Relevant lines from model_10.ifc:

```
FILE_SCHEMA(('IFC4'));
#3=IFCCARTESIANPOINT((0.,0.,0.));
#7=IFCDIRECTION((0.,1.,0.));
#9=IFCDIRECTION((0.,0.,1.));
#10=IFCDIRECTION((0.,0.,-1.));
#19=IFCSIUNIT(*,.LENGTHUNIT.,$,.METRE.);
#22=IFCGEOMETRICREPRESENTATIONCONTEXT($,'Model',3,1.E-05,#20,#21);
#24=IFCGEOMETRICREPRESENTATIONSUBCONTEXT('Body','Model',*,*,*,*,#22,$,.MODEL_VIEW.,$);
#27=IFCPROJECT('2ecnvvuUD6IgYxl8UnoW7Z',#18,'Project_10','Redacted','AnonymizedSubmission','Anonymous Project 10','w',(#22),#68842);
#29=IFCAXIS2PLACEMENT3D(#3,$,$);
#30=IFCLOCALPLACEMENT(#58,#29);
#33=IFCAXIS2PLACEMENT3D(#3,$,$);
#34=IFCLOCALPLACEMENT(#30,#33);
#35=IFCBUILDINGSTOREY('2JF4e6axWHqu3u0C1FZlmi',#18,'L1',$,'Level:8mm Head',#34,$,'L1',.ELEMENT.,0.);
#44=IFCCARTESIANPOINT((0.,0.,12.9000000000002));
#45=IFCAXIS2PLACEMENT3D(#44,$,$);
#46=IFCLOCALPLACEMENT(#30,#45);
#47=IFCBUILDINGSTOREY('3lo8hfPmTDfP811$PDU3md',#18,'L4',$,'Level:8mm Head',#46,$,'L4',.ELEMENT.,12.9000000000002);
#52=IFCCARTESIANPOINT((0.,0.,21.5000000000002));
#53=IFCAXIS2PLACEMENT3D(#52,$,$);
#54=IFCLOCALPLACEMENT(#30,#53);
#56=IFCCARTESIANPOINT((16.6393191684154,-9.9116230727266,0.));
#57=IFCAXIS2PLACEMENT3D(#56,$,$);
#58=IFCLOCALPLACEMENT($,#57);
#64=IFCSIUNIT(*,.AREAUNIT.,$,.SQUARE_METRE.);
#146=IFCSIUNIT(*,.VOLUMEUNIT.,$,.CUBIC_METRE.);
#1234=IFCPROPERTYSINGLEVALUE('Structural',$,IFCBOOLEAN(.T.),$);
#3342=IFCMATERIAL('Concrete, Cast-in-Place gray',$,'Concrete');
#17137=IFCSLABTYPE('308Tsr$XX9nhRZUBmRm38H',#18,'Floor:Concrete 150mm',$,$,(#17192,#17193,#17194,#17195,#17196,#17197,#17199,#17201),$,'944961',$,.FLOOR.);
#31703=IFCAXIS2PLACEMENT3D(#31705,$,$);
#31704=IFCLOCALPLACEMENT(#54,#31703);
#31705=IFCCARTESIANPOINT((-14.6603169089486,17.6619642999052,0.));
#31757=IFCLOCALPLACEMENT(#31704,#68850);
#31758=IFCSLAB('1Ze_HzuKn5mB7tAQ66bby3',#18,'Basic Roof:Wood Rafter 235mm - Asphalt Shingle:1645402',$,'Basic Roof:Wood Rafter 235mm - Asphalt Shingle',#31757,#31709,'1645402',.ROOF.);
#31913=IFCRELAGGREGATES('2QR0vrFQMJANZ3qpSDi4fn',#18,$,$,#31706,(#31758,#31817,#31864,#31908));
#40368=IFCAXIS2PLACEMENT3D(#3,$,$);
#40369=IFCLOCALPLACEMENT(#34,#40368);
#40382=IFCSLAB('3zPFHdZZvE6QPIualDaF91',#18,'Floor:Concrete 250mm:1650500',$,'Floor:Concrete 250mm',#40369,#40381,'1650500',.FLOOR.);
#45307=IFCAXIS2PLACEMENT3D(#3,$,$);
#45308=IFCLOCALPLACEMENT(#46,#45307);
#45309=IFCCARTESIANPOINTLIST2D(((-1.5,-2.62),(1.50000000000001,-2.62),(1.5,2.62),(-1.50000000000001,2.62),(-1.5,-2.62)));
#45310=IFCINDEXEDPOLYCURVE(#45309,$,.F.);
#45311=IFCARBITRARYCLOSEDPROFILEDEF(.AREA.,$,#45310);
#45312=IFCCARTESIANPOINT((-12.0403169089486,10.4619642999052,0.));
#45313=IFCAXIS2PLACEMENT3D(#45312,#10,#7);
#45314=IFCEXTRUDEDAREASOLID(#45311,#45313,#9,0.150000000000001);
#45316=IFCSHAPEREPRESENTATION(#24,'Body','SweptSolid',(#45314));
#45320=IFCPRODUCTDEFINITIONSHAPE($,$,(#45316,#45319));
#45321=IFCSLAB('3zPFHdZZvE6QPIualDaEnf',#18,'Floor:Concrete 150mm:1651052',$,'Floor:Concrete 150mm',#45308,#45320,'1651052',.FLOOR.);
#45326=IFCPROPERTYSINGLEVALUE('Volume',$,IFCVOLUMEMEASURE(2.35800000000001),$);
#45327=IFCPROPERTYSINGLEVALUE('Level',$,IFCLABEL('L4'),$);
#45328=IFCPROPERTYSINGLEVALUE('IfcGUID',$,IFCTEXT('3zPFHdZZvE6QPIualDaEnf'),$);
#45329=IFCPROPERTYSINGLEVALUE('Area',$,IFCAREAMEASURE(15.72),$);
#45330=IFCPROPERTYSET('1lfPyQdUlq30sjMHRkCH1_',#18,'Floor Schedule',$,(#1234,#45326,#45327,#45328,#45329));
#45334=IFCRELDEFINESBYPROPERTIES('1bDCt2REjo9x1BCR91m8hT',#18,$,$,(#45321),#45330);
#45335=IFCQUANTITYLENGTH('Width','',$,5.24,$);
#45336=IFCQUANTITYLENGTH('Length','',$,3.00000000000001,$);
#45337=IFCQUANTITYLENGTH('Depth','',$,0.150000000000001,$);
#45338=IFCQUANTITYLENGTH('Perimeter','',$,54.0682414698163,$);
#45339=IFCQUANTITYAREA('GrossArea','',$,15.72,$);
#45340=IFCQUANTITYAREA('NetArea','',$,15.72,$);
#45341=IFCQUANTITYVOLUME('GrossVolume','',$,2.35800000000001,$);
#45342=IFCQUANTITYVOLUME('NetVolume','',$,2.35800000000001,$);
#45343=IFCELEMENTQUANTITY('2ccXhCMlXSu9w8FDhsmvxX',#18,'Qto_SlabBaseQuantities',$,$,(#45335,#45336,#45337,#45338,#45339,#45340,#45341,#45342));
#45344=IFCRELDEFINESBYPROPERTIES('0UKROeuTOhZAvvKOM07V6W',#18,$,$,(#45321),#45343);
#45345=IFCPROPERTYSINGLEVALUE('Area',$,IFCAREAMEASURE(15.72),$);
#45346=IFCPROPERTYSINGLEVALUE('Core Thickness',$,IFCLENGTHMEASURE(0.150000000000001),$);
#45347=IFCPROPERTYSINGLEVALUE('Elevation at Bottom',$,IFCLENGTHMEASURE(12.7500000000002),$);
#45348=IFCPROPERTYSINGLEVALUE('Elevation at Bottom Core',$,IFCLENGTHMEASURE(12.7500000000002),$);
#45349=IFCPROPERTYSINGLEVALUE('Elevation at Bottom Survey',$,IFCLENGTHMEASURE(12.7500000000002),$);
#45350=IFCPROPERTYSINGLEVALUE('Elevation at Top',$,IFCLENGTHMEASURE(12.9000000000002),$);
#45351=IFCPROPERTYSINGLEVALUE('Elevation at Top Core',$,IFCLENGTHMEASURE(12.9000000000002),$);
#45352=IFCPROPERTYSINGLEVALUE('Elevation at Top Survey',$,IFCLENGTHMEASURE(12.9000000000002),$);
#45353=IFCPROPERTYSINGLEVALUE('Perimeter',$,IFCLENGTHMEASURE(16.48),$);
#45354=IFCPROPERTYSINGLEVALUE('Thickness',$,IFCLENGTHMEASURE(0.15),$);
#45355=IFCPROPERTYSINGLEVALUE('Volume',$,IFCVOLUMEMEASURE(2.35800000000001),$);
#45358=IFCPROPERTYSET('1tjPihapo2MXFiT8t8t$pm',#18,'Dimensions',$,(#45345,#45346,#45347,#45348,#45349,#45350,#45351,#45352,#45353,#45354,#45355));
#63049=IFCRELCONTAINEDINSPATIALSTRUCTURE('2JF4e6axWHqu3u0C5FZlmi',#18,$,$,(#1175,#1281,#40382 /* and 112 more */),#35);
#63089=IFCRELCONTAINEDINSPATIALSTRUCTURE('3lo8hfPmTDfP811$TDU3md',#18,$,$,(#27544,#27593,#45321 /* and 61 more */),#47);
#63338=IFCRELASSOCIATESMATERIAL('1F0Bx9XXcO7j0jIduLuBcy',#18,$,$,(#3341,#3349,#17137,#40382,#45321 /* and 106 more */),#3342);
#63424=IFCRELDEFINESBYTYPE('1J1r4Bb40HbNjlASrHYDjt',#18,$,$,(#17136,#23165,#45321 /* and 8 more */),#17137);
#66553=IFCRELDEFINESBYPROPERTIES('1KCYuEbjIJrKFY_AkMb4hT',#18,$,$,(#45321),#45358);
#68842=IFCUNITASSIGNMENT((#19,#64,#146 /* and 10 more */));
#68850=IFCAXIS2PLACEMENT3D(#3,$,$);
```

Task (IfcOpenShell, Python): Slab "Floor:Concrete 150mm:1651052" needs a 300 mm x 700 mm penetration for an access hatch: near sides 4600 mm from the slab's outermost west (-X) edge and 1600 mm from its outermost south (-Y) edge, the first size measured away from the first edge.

```python
import numpy as np
import ifcopenshell
import ifcopenshell.api.feature
import ifcopenshell.api.geometry
import ifcopenshell.api.pset
import ifcopenshell.api.root
import ifcopenshell.geom
import ifcopenshell.util.element
import ifcopenshell.util.placement
import ifcopenshell.util.representation
import ifcopenshell.util.shape
import ifcopenshell.util.unit

model = ifcopenshell.open("model_10.ifc")
unit_scale = ifcopenshell.util.unit.calculate_unit_scale(model)
area_scale = ifcopenshell.util.unit.calculate_unit_scale(model, "AREAUNIT")
volume_scale = ifcopenshell.util.unit.calculate_unit_scale(model, "VOLUMEUNIT")
settings = ifcopenshell.geom.settings()


def volume(element):
    """Net volume in cubic metres, openings subtracted."""
    shape = ifcopenshell.geom.create_shape(settings, element)
    return ifcopenshell.util.shape.get_volume(shape.geometry)


slab = model.by_guid("3zPFHdZZvE6QPIualDaEnf")
before = volume(slab)

# Extent in the slab's own axes, in metres. The edges named are its -X and -Y sides.
slab_shape = ifcopenshell.geom.create_shape(settings, slab)
vertices = ifcopenshell.util.shape.get_vertices(slab_shape.geometry)
x_min, y_min, bottom = vertices.min(axis=0)
top = vertices[:, 2].max()

opening = ifcopenshell.api.root.create_entity(model, ifc_class="IfcOpeningElement", name="Access hatch opening", predefined_type="OPENING")
context = ifcopenshell.util.representation.get_context(model, "Model", "Body", "MODEL_VIEW")
width, depth = 0.3, 0.7
outline = [(0.0, 0.0), (width, 0.0), (width, depth), (0.0, depth), (0.0, 0.0)]
# Overshoot both faces by 50 mm so the cut is clean.
shape = ifcopenshell.api.geometry.add_slab_representation(
    model, context=context, depth=top - bottom + 0.1, polyline=outline
)
ifcopenshell.api.geometry.assign_representation(model, product=opening, representation=shape)

matrix = ifcopenshell.util.placement.get_local_placement(slab.ObjectPlacement)
matrix[:, 3] = matrix @ np.append(np.array([x_min + 4.6, y_min + 1.6, bottom - 0.05]) / unit_scale, 1.0)
ifcopenshell.api.geometry.edit_object_placement(model, product=opening, matrix=matrix, is_si=False)
ifcopenshell.api.feature.add_feature(model, feature=opening, element=slab)

after = volume(slab)

# Update the slab's stored quantities.
pset = model.by_id(ifcopenshell.util.element.get_pset(slab, "Floor Schedule", should_inherit=False)["id"])
ifcopenshell.api.pset.edit_pset(model, pset=pset, properties={
    "Volume": model.create_entity("IfcVolumeMeasure", after / volume_scale),
    "Area": model.create_entity("IfcAreaMeasure", after / (top - bottom) / area_scale),
})
qto = model.by_id(ifcopenshell.util.element.get_pset(slab, "Qto_SlabBaseQuantities", should_inherit=False)["id"])
ifcopenshell.api.pset.edit_qto(model, qto=qto, properties={
    "NetArea": after / (top - bottom) / area_scale,
    "NetVolume": after / volume_scale,
})
pset = model.by_id(ifcopenshell.util.element.get_pset(slab, "Dimensions", should_inherit=False)["id"])
ifcopenshell.api.pset.edit_pset(model, pset=pset, properties={
    "Area": model.create_entity("IfcAreaMeasure", after / (top - bottom) / area_scale),
    "Volume": model.create_entity("IfcVolumeMeasure", after / volume_scale),
})

print(f"slab volume {before:.3f} -> {after:.3f} m3")

model.write("model_10-out.ifc")
```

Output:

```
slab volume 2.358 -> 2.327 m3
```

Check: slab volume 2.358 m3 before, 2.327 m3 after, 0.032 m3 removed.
